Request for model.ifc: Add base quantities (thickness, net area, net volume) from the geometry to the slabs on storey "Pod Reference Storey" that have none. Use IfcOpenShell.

First a look at what the model holds.

```python
import ifcopenshell
import ifcopenshell.util.element
import ifcopenshell.util.unit

model = ifcopenshell.open("model.ifc")
print(model.schema)
for unit_type in ("LENGTHUNIT", "AREAUNIT", "VOLUMEUNIT"):
    print(unit_type, ifcopenshell.util.unit.calculate_unit_scale(model, unit_type))
storey = next(s for s in model.by_type("IfcBuildingStorey") if s.Name == "Pod Reference Storey")
slabs = [e for e in ifcopenshell.util.element.get_decomposition(storey) if e.is_a("IfcSlab")]
for e in sorted(slabs, key=lambda e: e.id()):
    print(e.id(), e.is_a(), e.Name, list(ifcopenshell.util.element.get_psets(e, qtos_only=True)), sep=" | ")
```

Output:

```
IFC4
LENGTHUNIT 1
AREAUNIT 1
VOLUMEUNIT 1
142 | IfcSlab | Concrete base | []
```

```python
import ifcopenshell
import ifcopenshell.api.pset
import ifcopenshell.geom
import ifcopenshell.util.element
import ifcopenshell.util.shape
import ifcopenshell.util.unit

model = ifcopenshell.open("model.ifc")
unit_scale = ifcopenshell.util.unit.calculate_unit_scale(model)
area_scale = ifcopenshell.util.unit.calculate_unit_scale(model, "AREAUNIT")
volume_scale = ifcopenshell.util.unit.calculate_unit_scale(model, "VOLUMEUNIT")
settings = ifcopenshell.geom.settings()

storey = next(s for s in model.by_type("IfcBuildingStorey") if s.Name == "Pod Reference Storey")
slabs = [e for e in ifcopenshell.util.element.get_decomposition(storey) if e.is_a("IfcSlab")]

for e in sorted(slabs, key=lambda e: e.id()):
    if ifcopenshell.util.element.get_psets(e, qtos_only=True, should_inherit=False):
        continue
    # Geometry comes back in metres, in the element's own axes.
    shape = ifcopenshell.geom.create_shape(settings, e)
    values = {
        "Width": ifcopenshell.util.shape.get_z(shape.geometry) / unit_scale,
        "NetArea": ifcopenshell.util.shape.get_footprint_area(shape.geometry) / area_scale,
        "NetVolume": ifcopenshell.util.shape.get_volume(shape.geometry) / volume_scale,
    }
    qto = ifcopenshell.api.pset.add_qto(model, product=e, name="Qto_SlabBaseQuantities")
    ifcopenshell.api.pset.edit_qto(model, qto=qto, properties=values)
    print(e.id(), {k: round(v, 3) for k, v in values.items()})

model.write("model_edited.ifc")
```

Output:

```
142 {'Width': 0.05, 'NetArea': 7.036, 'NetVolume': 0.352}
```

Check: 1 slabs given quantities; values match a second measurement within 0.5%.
